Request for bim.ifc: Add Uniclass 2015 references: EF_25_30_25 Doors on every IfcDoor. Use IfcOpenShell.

First a look at what the model holds.

```python
import ifcopenshell

model = ifcopenshell.open("bim.ifc")
print(model.schema)
print("classifications:", [c.Name for c in model.by_type("IfcClassification")])
for ifc_class in ("IfcDoor", "IfcRoof", "IfcStair", "IfcWall", "IfcWindow"):
    print(ifc_class, len(model.by_type(ifc_class)))
```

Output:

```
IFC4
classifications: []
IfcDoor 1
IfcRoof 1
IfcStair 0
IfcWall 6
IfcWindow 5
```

```python
import ifcopenshell
import ifcopenshell.api.classification

model = ifcopenshell.open("bim.ifc")

system = ifcopenshell.api.classification.add_classification(model, classification="Uniclass 2015")

codes = {
    "IfcDoor": ("EF_25_30_25", "Doors"),
}
for ifc_class, (code, name) in codes.items():
    products = model.by_type(ifc_class)
    ifcopenshell.api.classification.add_reference(
        model, products=products, classification=system, identification=code, name=name
    )
    print(code, len(products))

model.write("bim-out.ifc")
```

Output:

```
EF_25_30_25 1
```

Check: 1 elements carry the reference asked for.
